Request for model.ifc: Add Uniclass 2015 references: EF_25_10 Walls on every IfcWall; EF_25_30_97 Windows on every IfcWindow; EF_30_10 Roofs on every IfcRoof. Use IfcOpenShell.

First a look at what the model holds.

```python
import ifcopenshell

model = ifcopenshell.open("model.ifc")
print(model.schema)
print("classifications:", [c.Name for c in model.by_type("IfcClassification")])
for ifc_class in ("IfcDoor", "IfcRoof", "IfcStair", "IfcWall", "IfcWindow"):
    print(ifc_class, len(model.by_type(ifc_class)))
```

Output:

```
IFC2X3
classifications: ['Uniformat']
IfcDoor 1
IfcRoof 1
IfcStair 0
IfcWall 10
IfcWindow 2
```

```python
import ifcopenshell
import ifcopenshell.api.classification

model = ifcopenshell.open("model.ifc")

# IFC2X3 requires Source and Edition and has no link from the project to the system.
system = model.create_entity("IfcClassification", Source="NBS", Edition="2015", Name="Uniclass 2015")

codes = {
    "IfcWall": ("EF_25_10", "Walls"),
    "IfcWindow": ("EF_25_30_97", "Windows"),
    "IfcRoof": ("EF_30_10", "Roofs"),
}
for ifc_class, (code, name) in codes.items():
    products = model.by_type(ifc_class)
    ifcopenshell.api.classification.add_reference(
        model, products=products, classification=system, identification=code, name=name
    )
    print(code, len(products))

model.write("model_updated.ifc")
```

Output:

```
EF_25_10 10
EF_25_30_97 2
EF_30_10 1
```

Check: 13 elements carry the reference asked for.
